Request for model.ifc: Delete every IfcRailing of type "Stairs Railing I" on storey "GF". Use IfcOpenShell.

First a look at what the model holds.

```python
import ifcopenshell
import ifcopenshell.util.element

model = ifcopenshell.open("model.ifc")
print(model.schema)
storey = next(s for s in model.by_type("IfcBuildingStorey") if s.Name == "GF")
railings = [e for e in ifcopenshell.util.element.get_decomposition(storey) if e.is_a("IfcRailing")]
seen = {}
for e in railings:
    element_type = ifcopenshell.util.element.get_type(e)
    name = element_type.Name if element_type not in (None, e) else None
    seen[name] = seen.get(name, 0) + 1
for name, count in sorted(seen.items(), key=str):
    print(count, "x", name)
```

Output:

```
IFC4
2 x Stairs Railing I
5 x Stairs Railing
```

```python
import ifcopenshell
import ifcopenshell.api.root
import ifcopenshell.util.element

model = ifcopenshell.open("model.ifc")

storey = next(s for s in model.by_type("IfcBuildingStorey") if s.Name == "GF")
railings = [e for e in ifcopenshell.util.element.get_decomposition(storey) if e.is_a("IfcRailing")]
targets = [e for e in railings if (t := ifcopenshell.util.element.get_type(e)) not in (None, e) and t.Name == "Stairs Railing I"]

for e in targets:
    ifcopenshell.api.root.remove_product(model, product=e)
print(len(targets), "removed")

model.write("model_updated.ifc")
```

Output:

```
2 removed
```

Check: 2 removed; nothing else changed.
